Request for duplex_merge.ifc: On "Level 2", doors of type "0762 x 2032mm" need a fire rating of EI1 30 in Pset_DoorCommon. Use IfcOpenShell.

First a look at what the model holds.

```python
import ifcopenshell
import ifcopenshell.util.element

model = ifcopenshell.open("duplex_merge.ifc")
print(model.schema)
storey = next(s for s in model.by_type("IfcBuildingStorey") if s.Name == "Level 2")
doors = [e for e in ifcopenshell.util.element.get_decomposition(storey) if e.is_a("IfcDoor")]
seen = {}
for e in doors:
    element_type = ifcopenshell.util.element.get_type(e)
    key = (element_type.Name if element_type != e and element_type else None, ifcopenshell.util.element.get_pset(e, "Pset_DoorCommon", "FireRating"))
    seen[key] = seen.get(key, 0) + 1
for (name, value), count in sorted(seen.items(), key=str):
    print(count, "x", name, "|", value)
```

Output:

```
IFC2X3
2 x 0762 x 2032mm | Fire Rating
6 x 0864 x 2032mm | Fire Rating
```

```python
import ifcopenshell
import ifcopenshell.api.pset
import ifcopenshell.util.element

model = ifcopenshell.open("duplex_merge.ifc")

storey = next(s for s in model.by_type("IfcBuildingStorey") if s.Name == "Level 2")
doors = [e for e in ifcopenshell.util.element.get_decomposition(storey) if e.is_a("IfcDoor")]

count = 0
for e in doors:
    element_type = ifcopenshell.util.element.get_type(e)
    if element_type in (None, e) or element_type.Name != "0762 x 2032mm":
        continue
    # add_pset returns the element's existing set when there is one.
    pset = ifcopenshell.api.pset.add_pset(model, product=e, name="Pset_DoorCommon")
    ifcopenshell.api.pset.edit_pset(model, pset=pset, properties={"FireRating": "EI1 30"})
    count += 1

print(count, "doors updated")

model.write("duplex_merge-out.ifc")
```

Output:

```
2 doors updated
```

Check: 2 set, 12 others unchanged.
